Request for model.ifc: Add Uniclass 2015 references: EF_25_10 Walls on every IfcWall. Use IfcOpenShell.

First a look at what the model holds.

```python
import ifcopenshell

model = ifcopenshell.open("model.ifc")
print(model.schema)
print("classifications:", [c.Name for c in model.by_type("IfcClassification")])
for ifc_class in ("IfcDoor", "IfcRoof", "IfcStair", "IfcWall", "IfcWindow"):
    print(ifc_class, len(model.by_type(ifc_class)))
```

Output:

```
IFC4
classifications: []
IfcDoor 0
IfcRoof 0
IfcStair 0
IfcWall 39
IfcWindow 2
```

```python
import ifcopenshell
import ifcopenshell.api.classification

model = ifcopenshell.open("model.ifc")

system = ifcopenshell.api.classification.add_classification(model, classification="Uniclass 2015")

codes = {
    "IfcWall": ("EF_25_10", "Walls"),
}
for ifc_class, (code, name) in codes.items():
    products = model.by_type(ifc_class)
    ifcopenshell.api.classification.add_reference(
        model, products=products, classification=system, identification=code, name=name
    )
    print(code, len(products))

model.write("model_updated.ifc")
```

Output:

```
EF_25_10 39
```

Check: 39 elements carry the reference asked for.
